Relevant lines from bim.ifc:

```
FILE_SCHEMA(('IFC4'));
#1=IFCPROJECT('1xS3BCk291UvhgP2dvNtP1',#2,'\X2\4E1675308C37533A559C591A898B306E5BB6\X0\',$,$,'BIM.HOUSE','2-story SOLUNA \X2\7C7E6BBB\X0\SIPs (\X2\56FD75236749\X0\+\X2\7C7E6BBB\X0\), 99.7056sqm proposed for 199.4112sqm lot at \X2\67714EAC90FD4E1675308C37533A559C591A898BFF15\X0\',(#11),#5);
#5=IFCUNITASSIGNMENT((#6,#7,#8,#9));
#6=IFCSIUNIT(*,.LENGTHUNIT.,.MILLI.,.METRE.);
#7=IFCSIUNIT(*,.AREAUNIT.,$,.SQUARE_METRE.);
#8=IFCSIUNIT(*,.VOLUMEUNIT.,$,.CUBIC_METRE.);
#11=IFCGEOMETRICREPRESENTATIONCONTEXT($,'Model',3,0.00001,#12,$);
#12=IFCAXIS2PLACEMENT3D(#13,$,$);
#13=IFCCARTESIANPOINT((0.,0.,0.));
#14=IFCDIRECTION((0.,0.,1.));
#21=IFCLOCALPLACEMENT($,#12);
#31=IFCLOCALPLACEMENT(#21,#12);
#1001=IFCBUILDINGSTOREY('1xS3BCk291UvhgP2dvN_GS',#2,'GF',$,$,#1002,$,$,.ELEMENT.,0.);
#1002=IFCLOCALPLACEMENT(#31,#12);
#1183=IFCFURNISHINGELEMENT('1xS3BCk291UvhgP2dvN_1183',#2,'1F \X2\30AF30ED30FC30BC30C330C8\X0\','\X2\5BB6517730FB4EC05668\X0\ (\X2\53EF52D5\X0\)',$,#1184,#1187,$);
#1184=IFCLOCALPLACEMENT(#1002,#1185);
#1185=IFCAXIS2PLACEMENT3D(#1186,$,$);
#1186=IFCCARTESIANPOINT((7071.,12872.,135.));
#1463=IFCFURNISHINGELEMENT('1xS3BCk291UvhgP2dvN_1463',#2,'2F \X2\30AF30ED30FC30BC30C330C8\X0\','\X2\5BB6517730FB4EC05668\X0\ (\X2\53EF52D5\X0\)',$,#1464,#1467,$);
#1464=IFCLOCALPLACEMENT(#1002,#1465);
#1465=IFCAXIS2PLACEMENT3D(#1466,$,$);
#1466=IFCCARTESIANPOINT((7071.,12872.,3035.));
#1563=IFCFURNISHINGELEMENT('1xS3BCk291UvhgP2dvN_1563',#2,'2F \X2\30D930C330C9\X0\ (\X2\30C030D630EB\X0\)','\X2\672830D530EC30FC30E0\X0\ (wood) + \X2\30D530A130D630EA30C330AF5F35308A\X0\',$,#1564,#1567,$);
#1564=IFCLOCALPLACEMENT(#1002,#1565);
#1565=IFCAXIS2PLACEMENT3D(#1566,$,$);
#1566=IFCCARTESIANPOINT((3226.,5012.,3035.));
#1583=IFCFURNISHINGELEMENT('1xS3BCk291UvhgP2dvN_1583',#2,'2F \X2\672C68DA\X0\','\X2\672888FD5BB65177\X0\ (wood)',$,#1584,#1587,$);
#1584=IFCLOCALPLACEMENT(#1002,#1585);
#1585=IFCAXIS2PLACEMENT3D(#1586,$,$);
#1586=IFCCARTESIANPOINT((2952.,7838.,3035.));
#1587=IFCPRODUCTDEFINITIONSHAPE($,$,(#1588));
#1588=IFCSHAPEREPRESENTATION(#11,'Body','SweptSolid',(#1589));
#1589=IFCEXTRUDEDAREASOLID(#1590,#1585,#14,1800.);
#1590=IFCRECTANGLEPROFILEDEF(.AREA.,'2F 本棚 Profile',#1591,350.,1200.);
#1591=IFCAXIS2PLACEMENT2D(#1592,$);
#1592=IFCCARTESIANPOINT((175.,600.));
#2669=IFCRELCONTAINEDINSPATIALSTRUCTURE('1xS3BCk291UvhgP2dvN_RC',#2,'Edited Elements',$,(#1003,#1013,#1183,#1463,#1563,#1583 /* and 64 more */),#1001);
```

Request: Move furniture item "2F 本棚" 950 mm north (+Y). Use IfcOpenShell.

```python
import ifcopenshell
import ifcopenshell.api.geometry
import ifcopenshell.util.placement
import ifcopenshell.util.unit

model = ifcopenshell.open("bim.ifc")
unit_scale = ifcopenshell.util.unit.calculate_unit_scale(model)

item = model.by_guid("1xS3BCk291UvhgP2dvN_1583")
matrix = ifcopenshell.util.placement.get_local_placement(item.ObjectPlacement)
matrix[1, 3] += 0.95 / unit_scale
ifcopenshell.api.geometry.edit_object_placement(model, product=item, matrix=matrix, is_si=False)

print(ifcopenshell.util.placement.get_local_placement(item.ObjectPlacement).round(3) + 0.0)

model.write("bim_v2.ifc")
```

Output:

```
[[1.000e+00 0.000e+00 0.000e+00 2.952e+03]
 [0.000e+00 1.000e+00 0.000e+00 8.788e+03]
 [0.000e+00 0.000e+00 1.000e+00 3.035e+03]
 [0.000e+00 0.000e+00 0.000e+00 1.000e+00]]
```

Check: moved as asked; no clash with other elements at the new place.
